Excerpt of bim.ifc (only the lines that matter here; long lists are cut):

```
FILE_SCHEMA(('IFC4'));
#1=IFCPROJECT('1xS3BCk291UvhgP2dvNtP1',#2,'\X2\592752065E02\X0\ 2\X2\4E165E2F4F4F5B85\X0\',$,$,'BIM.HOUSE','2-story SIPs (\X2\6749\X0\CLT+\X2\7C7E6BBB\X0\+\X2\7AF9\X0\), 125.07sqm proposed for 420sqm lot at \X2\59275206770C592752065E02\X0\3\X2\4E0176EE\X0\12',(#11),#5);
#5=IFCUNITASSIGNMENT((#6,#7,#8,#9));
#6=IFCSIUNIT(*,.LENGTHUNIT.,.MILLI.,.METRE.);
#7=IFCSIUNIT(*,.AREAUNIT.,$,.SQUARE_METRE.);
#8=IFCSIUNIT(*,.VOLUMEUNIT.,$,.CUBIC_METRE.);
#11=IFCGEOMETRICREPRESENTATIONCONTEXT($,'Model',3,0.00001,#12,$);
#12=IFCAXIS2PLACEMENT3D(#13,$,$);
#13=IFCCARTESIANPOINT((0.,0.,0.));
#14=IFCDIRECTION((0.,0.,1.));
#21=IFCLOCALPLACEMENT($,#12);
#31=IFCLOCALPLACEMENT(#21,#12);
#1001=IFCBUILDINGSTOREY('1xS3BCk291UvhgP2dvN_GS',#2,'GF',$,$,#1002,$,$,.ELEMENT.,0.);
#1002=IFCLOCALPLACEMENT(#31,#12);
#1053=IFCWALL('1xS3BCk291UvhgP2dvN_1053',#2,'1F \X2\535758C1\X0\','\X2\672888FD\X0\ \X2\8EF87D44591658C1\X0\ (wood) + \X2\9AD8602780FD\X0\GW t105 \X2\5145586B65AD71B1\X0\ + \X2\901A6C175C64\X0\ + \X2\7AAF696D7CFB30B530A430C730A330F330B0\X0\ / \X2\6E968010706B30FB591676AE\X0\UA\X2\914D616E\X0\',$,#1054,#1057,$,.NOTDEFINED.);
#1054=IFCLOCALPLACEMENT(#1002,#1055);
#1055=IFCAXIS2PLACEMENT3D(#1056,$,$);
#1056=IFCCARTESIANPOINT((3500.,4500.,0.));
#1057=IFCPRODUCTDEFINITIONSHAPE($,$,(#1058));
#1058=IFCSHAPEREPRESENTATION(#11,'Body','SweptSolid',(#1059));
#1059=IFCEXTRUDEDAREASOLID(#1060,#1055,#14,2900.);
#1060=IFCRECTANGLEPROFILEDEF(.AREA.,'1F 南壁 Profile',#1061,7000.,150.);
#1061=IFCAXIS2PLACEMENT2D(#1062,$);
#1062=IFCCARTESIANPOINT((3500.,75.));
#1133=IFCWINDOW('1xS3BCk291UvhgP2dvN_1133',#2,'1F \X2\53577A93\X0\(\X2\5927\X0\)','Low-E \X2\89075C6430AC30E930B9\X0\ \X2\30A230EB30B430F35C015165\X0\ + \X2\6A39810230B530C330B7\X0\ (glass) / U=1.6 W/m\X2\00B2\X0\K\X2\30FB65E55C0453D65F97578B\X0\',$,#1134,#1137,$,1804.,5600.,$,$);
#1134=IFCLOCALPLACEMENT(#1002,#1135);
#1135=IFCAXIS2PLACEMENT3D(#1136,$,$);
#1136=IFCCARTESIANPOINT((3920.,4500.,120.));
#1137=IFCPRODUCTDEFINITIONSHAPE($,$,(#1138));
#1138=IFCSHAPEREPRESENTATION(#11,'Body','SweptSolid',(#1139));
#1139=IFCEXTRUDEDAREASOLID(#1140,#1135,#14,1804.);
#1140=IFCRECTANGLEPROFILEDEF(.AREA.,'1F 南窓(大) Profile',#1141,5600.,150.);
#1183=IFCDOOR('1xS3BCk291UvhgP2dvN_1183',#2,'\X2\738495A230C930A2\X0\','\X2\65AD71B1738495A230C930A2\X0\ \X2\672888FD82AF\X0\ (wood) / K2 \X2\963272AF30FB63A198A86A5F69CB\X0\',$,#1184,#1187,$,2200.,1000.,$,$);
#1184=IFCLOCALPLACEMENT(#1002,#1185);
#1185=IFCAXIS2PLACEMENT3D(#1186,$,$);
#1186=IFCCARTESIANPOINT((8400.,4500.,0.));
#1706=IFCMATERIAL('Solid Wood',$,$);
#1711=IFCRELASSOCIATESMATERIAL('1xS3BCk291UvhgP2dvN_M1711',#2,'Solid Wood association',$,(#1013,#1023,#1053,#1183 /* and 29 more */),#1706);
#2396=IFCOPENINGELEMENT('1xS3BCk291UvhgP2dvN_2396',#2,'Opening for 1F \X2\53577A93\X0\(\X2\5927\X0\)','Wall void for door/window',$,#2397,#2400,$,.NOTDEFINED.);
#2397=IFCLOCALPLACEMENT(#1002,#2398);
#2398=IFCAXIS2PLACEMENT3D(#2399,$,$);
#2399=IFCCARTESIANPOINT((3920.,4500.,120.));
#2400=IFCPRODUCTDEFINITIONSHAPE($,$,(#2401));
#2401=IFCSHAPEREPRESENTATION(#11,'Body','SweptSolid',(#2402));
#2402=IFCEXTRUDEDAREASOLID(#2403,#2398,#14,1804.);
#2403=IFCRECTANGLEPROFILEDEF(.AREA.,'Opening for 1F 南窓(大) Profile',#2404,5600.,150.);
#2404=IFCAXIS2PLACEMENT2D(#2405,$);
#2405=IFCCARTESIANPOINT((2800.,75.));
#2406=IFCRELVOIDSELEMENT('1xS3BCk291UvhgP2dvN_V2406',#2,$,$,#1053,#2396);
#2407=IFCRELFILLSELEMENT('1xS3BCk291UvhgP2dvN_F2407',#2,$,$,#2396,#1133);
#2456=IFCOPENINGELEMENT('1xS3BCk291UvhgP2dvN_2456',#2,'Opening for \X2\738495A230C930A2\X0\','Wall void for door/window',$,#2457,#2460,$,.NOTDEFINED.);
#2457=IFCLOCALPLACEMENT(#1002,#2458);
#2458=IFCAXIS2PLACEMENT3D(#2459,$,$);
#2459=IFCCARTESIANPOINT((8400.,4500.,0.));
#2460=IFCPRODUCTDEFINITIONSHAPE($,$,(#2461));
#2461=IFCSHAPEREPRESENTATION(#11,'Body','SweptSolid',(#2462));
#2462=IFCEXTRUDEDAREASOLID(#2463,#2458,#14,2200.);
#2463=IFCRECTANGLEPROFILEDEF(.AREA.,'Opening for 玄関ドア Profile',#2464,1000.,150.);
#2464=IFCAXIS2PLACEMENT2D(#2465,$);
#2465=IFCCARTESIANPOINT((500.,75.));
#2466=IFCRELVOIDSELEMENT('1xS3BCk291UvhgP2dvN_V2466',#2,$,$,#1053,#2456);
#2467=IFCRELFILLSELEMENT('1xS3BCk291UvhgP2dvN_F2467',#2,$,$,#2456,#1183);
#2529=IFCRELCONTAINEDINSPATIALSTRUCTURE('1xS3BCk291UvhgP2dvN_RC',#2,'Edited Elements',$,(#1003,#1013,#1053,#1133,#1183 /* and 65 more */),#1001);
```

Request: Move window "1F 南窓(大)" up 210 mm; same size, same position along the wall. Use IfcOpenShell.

```python
import numpy as np
import ifcopenshell
import ifcopenshell.api.geometry
import ifcopenshell.util.placement
import ifcopenshell.util.unit

model = ifcopenshell.open("bim.ifc")
unit_scale = ifcopenshell.util.unit.calculate_unit_scale(model)

window = model.by_guid("1xS3BCk291UvhgP2dvN_1133")
opening = window.FillsVoids[0].RelatingOpeningElement
dz = 0.21 / unit_scale

shift = np.array([0.0, 0.0, dz])
# The window is not placed relative to its opening, so move both.
for product in (opening, window):
    matrix = ifcopenshell.util.placement.get_local_placement(product.ObjectPlacement)
    matrix[:3, 3] += shift
    ifcopenshell.api.geometry.edit_object_placement(model, product=product, matrix=matrix, is_si=False)

print(f"moved by {dz * unit_scale:+.3f} m")

model.write("bim_rev.ifc")
```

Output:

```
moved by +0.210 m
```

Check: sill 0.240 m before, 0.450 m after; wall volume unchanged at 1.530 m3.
